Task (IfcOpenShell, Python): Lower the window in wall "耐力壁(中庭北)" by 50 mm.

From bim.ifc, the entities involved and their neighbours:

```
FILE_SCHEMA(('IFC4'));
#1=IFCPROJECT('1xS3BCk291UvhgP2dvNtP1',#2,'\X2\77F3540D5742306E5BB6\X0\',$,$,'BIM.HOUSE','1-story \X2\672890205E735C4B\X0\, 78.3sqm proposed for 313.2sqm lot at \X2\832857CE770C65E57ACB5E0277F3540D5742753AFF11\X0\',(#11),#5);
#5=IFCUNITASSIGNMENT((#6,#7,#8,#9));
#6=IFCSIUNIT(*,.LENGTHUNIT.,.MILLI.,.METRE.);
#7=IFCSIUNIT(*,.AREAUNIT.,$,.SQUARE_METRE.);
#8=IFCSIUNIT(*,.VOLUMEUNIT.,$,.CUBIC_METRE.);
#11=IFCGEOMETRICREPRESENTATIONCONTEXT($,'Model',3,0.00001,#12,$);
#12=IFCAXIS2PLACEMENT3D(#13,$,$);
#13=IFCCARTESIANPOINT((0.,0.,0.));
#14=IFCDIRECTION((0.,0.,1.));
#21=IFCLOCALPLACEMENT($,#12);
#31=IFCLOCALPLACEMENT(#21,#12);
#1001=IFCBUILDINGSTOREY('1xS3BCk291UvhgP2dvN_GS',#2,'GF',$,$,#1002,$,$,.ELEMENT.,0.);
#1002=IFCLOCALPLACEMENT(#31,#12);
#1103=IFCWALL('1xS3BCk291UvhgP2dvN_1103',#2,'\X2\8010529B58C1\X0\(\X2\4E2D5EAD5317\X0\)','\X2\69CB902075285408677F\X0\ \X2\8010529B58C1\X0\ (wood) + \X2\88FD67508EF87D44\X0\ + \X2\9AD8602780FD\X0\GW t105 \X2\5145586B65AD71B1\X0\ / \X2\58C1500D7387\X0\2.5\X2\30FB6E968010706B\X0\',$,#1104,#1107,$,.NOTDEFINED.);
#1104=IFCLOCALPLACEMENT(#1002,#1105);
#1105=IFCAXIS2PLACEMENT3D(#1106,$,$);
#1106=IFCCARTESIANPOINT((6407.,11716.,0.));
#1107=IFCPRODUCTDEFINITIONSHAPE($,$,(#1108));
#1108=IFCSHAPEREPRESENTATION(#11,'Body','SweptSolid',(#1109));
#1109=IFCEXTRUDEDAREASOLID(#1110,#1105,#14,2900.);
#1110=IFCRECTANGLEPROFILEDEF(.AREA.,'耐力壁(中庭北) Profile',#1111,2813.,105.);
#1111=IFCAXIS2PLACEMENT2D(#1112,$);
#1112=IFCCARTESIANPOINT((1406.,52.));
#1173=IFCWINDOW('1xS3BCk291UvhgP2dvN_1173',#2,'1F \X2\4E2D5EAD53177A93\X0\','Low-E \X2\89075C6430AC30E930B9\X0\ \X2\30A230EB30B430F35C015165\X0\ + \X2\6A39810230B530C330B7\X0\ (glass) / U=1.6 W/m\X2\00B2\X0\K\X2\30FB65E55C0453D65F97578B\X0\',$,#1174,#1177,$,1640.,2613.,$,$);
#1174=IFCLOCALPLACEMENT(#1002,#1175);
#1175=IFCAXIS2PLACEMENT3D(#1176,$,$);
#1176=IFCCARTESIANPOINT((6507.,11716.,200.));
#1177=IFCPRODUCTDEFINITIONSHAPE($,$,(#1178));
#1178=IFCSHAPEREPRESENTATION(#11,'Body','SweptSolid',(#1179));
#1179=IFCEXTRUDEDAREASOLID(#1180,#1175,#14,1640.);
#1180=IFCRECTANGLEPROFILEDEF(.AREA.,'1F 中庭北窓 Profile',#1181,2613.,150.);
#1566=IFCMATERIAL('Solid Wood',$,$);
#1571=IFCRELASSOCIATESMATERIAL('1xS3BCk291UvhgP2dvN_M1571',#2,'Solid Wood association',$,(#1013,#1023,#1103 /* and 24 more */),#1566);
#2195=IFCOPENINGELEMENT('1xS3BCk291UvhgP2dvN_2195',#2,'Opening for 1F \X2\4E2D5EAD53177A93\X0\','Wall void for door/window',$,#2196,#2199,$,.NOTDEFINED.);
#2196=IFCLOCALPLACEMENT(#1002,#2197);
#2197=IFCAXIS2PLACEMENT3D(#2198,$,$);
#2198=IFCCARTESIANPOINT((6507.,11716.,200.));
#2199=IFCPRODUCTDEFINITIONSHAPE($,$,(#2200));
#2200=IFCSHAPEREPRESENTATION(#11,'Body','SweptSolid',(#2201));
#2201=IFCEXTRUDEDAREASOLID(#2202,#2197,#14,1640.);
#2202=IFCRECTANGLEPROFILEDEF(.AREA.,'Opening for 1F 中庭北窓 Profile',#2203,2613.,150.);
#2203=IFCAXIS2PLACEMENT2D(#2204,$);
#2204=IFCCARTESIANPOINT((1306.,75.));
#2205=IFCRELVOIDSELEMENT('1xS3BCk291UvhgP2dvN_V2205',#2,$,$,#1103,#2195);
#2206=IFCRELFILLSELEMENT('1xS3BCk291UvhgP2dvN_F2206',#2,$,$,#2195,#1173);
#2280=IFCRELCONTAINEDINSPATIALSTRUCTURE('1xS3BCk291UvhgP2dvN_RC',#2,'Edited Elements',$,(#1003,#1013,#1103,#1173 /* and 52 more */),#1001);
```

```python
import numpy as np
import ifcopenshell
import ifcopenshell.api.geometry
import ifcopenshell.util.placement
import ifcopenshell.util.unit

model = ifcopenshell.open("bim.ifc")
unit_scale = ifcopenshell.util.unit.calculate_unit_scale(model)

window = model.by_id(1173)
opening = window.FillsVoids[0].RelatingOpeningElement
dz = -0.05 / unit_scale

shift = np.array([0.0, 0.0, dz])
# The window is not placed relative to its opening, so move both.
for product in (opening, window):
    matrix = ifcopenshell.util.placement.get_local_placement(product.ObjectPlacement)
    matrix[:3, 3] += shift
    ifcopenshell.api.geometry.edit_object_placement(model, product=product, matrix=matrix, is_si=False)

print(f"moved by {dz * unit_scale:+.3f} m")

model.write("bim_edited.ifc")
```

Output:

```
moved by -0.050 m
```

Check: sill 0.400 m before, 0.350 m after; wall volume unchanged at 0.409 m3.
